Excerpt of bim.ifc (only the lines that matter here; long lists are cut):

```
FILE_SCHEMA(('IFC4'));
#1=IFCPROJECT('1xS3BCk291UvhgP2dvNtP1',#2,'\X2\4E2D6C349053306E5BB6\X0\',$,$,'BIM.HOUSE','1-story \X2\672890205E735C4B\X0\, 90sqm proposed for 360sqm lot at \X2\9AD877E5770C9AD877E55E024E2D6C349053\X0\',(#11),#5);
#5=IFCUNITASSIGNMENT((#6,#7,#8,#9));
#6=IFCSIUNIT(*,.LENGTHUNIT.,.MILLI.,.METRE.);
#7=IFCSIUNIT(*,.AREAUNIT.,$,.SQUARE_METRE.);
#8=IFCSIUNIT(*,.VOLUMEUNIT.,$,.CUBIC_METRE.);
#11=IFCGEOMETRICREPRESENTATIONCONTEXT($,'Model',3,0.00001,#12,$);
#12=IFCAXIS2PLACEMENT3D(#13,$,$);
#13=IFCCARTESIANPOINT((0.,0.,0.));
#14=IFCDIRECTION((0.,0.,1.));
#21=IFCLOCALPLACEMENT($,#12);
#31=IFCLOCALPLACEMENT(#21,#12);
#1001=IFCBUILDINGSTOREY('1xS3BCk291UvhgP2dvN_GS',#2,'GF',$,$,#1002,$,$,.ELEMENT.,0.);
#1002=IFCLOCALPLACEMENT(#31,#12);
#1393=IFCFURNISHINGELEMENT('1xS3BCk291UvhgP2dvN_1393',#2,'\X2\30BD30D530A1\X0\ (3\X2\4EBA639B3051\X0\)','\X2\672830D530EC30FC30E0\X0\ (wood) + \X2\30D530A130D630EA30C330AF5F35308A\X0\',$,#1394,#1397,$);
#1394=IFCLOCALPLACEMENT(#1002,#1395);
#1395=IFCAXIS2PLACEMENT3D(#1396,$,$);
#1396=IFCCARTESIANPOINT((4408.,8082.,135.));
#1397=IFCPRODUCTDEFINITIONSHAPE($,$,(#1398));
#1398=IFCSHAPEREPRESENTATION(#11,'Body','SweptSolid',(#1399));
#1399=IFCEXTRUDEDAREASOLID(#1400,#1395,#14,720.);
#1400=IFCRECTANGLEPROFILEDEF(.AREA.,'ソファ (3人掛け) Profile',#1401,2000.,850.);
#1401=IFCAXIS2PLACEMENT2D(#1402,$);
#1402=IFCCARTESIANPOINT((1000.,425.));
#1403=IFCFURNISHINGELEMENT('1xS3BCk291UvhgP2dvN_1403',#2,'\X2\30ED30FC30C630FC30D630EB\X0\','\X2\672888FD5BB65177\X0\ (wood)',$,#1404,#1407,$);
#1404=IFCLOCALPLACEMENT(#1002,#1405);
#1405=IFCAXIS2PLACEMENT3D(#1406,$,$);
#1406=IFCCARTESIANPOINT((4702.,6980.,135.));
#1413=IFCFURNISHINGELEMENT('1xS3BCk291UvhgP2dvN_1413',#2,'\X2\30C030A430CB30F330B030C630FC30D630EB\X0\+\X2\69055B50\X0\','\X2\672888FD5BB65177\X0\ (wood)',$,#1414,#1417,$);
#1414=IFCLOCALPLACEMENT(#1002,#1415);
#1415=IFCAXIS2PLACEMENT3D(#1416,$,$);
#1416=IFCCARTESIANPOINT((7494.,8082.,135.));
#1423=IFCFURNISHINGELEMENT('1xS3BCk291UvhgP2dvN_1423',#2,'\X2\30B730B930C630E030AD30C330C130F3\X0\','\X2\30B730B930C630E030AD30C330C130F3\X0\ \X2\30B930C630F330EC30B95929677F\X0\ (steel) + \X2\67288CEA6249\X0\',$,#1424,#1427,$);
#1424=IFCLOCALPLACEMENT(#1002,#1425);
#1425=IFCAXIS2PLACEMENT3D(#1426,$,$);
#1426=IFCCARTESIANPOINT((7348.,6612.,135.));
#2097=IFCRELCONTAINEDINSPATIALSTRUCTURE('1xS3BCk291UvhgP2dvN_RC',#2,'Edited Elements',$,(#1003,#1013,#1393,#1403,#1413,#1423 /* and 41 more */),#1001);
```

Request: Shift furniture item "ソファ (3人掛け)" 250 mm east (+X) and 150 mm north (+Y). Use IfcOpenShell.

```python
import ifcopenshell
import ifcopenshell.api.geometry
import ifcopenshell.util.placement
import ifcopenshell.util.unit

model = ifcopenshell.open("bim.ifc")
unit_scale = ifcopenshell.util.unit.calculate_unit_scale(model)

item = model.by_guid("1xS3BCk291UvhgP2dvN_1393")
matrix = ifcopenshell.util.placement.get_local_placement(item.ObjectPlacement)
matrix[0, 3] += 0.25 / unit_scale
matrix[1, 3] += 0.15 / unit_scale
ifcopenshell.api.geometry.edit_object_placement(model, product=item, matrix=matrix, is_si=False)

print(ifcopenshell.util.placement.get_local_placement(item.ObjectPlacement).round(3) + 0.0)

model.write("bim-out.ifc")
```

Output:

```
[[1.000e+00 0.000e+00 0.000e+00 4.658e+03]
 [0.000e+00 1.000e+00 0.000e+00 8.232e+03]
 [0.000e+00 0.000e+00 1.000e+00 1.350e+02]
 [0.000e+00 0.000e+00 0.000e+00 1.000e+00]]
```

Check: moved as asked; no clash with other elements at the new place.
